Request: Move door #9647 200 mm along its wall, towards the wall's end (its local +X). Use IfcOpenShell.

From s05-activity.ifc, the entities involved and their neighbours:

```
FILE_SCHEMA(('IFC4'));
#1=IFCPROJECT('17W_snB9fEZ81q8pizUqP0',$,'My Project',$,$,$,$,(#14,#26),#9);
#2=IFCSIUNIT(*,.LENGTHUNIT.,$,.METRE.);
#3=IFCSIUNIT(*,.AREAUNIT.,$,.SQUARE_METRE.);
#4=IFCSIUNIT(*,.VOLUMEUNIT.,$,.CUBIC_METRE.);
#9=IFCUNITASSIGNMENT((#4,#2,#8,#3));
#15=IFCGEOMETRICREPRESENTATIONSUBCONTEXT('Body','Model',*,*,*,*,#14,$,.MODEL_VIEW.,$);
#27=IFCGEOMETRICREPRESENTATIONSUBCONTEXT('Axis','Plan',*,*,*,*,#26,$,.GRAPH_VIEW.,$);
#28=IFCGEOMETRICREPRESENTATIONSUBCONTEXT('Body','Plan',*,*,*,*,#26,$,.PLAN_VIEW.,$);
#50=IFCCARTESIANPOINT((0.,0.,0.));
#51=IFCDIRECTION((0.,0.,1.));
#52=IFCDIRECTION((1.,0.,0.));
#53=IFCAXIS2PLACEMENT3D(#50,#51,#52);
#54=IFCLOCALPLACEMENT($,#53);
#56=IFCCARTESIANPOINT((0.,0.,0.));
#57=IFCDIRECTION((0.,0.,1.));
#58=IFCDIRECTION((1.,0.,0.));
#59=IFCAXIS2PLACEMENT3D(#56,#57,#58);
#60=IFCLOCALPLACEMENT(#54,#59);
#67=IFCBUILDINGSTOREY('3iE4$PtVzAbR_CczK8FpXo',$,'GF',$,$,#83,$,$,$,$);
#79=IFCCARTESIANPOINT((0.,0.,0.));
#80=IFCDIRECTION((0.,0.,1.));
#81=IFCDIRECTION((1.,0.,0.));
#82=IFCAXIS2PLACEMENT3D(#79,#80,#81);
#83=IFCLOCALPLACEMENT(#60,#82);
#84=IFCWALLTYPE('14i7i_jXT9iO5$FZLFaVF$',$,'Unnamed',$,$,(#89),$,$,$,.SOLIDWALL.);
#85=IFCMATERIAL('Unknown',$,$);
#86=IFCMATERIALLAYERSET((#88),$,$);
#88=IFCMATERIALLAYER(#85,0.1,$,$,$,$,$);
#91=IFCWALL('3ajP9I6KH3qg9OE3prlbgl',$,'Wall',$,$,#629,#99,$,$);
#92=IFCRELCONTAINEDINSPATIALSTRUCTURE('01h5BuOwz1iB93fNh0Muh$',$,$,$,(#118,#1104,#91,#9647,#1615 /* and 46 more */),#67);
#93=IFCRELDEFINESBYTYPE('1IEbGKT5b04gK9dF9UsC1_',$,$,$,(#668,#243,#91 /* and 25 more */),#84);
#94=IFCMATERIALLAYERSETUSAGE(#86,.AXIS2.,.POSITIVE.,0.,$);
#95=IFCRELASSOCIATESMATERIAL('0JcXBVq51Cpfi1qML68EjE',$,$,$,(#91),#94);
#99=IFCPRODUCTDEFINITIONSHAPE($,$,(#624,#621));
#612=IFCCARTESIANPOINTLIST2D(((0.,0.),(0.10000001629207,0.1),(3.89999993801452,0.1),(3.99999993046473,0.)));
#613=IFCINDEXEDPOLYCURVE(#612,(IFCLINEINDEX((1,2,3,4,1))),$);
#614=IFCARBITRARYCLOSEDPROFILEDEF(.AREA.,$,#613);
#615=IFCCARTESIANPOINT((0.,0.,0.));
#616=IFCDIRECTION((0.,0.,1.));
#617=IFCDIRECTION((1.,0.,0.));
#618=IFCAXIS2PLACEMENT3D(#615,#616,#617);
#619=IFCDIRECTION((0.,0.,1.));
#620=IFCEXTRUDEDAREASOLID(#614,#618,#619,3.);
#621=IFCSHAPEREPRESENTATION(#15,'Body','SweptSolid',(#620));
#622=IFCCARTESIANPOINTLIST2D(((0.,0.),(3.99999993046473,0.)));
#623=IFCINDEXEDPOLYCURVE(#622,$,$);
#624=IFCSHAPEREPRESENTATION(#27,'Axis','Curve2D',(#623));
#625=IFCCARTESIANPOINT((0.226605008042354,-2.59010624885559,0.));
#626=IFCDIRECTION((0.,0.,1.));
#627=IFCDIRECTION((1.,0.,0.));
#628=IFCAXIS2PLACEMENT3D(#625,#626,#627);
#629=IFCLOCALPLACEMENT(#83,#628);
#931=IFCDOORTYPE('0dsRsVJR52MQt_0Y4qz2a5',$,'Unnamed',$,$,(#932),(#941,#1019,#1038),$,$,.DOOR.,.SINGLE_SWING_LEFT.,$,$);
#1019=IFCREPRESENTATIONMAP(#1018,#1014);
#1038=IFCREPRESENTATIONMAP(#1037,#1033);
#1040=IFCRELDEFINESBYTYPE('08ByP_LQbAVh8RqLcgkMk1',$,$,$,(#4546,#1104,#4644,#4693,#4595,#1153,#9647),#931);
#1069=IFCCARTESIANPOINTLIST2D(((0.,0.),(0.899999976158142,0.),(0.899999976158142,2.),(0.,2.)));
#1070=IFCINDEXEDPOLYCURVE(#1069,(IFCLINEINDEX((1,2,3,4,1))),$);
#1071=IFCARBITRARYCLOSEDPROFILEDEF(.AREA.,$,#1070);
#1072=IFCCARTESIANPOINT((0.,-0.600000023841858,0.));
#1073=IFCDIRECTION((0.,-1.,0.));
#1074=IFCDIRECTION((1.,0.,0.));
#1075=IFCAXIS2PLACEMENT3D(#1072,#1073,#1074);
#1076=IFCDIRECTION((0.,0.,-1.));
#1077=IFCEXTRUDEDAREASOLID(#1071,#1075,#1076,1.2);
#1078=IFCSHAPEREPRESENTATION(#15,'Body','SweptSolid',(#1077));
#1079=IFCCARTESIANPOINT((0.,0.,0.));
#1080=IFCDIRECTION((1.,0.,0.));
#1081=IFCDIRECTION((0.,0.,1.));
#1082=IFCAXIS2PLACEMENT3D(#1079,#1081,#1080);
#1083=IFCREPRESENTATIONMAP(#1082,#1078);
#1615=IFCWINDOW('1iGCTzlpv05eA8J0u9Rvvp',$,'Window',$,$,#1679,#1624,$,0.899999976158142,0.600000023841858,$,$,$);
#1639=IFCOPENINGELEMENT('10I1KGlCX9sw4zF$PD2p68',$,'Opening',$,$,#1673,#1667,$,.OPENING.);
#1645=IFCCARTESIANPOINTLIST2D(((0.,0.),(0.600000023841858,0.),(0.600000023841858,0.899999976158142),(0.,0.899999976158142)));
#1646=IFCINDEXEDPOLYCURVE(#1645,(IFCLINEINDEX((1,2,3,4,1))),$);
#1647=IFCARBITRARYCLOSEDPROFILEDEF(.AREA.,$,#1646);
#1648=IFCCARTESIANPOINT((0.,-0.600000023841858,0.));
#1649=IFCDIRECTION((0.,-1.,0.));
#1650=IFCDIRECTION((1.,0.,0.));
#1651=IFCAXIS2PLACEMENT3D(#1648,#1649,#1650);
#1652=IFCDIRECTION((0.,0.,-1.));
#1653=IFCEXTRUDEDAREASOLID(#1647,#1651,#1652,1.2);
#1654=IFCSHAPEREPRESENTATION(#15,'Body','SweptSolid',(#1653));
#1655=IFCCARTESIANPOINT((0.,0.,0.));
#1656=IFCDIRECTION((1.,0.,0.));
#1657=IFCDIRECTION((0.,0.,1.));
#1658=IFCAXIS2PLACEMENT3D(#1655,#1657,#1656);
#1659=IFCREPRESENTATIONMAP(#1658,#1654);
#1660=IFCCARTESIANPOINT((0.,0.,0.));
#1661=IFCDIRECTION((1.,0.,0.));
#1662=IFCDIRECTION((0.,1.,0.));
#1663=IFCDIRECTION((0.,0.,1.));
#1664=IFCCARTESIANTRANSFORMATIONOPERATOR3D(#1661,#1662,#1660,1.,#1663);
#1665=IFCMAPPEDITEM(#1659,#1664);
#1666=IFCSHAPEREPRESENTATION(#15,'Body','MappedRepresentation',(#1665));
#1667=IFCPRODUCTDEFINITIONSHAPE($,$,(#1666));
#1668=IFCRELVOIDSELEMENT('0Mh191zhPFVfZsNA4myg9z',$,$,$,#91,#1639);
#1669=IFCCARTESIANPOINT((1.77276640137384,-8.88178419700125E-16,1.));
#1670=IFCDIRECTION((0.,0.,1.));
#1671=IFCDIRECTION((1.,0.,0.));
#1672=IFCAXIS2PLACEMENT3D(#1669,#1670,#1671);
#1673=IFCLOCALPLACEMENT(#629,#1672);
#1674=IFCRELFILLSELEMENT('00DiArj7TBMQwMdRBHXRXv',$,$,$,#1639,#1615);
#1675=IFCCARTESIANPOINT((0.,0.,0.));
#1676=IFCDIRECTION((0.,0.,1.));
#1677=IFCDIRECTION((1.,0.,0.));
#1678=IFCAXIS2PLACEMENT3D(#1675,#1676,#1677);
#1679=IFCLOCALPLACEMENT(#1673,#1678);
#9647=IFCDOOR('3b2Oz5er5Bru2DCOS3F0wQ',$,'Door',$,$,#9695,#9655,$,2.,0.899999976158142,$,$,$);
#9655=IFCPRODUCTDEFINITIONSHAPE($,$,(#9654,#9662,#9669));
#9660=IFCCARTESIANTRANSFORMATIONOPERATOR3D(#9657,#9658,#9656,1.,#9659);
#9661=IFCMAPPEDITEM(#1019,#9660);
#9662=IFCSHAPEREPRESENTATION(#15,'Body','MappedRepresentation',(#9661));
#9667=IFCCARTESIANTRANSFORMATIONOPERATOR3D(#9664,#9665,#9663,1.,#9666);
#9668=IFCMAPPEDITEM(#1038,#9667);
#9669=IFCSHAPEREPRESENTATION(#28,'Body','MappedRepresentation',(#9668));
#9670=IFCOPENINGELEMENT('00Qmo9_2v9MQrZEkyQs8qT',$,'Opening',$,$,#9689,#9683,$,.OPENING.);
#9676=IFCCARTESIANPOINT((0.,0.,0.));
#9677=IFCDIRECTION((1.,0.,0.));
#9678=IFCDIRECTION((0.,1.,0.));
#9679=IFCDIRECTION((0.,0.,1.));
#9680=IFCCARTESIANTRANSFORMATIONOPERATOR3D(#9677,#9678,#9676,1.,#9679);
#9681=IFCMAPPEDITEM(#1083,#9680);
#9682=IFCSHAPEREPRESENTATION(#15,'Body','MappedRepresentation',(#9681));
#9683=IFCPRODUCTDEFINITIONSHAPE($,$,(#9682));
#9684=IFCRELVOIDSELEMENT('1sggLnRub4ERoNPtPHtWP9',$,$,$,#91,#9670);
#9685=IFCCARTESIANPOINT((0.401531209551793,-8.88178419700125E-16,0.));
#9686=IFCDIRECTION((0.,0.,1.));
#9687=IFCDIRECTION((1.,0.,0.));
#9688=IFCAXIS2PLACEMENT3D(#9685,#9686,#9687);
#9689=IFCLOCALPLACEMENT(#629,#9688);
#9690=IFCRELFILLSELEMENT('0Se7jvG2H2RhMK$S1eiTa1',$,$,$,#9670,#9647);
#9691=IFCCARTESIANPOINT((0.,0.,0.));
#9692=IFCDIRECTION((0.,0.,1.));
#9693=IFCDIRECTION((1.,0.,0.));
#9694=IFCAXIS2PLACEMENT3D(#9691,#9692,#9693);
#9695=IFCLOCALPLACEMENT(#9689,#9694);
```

```python
import ifcopenshell
import ifcopenshell.api.geometry
import ifcopenshell.util.placement

model = ifcopenshell.open("s05-activity.ifc")

door = model.by_guid("3b2Oz5er5Bru2DCOS3F0wQ")
opening = door.FillsVoids[0].RelatingOpeningElement
wall = opening.VoidsElements[0].RelatingBuildingElement

wall_matrix = ifcopenshell.util.placement.get_local_placement(wall.ObjectPlacement)
shift = wall_matrix[:3, 0] * 0.2
before = ifcopenshell.util.placement.get_local_placement(door.ObjectPlacement)[:3, 3].copy()

# The door is placed relative to its opening, so it follows when the opening moves.
matrix = ifcopenshell.util.placement.get_local_placement(opening.ObjectPlacement)
matrix[:3, 3] += shift
ifcopenshell.api.geometry.edit_object_placement(
    model, product=opening, matrix=matrix, is_si=False, should_transform_children=True
)

after = ifcopenshell.util.placement.get_local_placement(door.ObjectPlacement)[:3, 3]
print("door moved by", (after - before).round(3) + 0.0)

model.write("s05-activity-out.ifc")
```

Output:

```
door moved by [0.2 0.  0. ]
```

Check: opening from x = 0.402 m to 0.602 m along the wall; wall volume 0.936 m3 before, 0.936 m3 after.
